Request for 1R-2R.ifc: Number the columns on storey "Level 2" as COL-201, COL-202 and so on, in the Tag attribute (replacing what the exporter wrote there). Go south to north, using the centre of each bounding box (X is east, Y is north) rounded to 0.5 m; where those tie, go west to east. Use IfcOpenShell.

First a look at what the model holds.

```python
import ifcopenshell
import ifcopenshell.util.element
import ifcopenshell.util.placement

model = ifcopenshell.open("1R-2R.ifc")
print(model.schema)
storey = next(s for s in model.by_type("IfcBuildingStorey") if s.Name == "Level 2")
columns = [e for e in ifcopenshell.util.element.get_decomposition(storey) if e.is_a("IfcColumn")]
for e in sorted(columns, key=lambda e: e.id()):
    origin = ifcopenshell.util.placement.get_local_placement(e.ObjectPlacement)[:3, 3]
    print(e.id(), e.Tag, e.Name, origin.round(2) + 0.0, sep=" | ")
```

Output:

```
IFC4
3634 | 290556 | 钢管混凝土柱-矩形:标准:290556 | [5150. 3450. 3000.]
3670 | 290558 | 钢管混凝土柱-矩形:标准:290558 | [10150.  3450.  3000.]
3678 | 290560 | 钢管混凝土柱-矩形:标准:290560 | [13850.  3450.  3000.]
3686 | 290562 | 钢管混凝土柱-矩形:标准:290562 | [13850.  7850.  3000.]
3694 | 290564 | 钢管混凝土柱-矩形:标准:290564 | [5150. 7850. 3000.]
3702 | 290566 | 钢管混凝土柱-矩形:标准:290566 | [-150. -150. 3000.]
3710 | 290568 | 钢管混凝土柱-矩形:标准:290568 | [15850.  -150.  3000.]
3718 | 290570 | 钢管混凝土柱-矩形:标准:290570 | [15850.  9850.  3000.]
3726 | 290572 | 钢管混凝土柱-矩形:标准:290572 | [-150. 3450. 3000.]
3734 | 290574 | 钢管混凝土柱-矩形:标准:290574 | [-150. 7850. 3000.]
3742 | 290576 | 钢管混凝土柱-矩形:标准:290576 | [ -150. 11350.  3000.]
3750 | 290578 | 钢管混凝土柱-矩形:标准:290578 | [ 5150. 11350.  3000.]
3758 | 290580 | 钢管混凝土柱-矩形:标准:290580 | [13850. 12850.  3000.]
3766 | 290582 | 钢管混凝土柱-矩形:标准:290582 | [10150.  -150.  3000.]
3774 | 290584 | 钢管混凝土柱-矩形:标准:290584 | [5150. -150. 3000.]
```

```python
import ifcopenshell
import ifcopenshell.geom
import ifcopenshell.util.element
import ifcopenshell.util.shape

model = ifcopenshell.open("1R-2R.ifc")
settings = ifcopenshell.geom.settings()
settings.set("use-world-coords", True)


def centre(element):
    shape = ifcopenshell.geom.create_shape(settings, element)
    return ifcopenshell.util.shape.get_bbox_centroid(shape.geometry)


storey = next(s for s in model.by_type("IfcBuildingStorey") if s.Name == "Level 2")
columns = [e for e in ifcopenshell.util.element.get_decomposition(storey) if e.is_a("IfcColumn")]

# Insertion points can sit at a corner or the storey origin, so sort by the geometry (in metres).
centres = {e: centre(e) for e in columns}
columns.sort(key=lambda e: (round(centres[e][1] / 0.5), centres[e][0]))

for i, e in enumerate(columns, start=1):
    number = f"COL-2{i:02d}"
    e.Tag = number
    print(e.id(), number)

model.write("1R-2R_edited.ifc")
```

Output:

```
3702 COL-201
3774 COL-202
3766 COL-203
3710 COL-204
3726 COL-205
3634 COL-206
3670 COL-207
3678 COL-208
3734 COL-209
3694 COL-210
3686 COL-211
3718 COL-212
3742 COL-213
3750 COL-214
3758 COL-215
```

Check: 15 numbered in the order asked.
